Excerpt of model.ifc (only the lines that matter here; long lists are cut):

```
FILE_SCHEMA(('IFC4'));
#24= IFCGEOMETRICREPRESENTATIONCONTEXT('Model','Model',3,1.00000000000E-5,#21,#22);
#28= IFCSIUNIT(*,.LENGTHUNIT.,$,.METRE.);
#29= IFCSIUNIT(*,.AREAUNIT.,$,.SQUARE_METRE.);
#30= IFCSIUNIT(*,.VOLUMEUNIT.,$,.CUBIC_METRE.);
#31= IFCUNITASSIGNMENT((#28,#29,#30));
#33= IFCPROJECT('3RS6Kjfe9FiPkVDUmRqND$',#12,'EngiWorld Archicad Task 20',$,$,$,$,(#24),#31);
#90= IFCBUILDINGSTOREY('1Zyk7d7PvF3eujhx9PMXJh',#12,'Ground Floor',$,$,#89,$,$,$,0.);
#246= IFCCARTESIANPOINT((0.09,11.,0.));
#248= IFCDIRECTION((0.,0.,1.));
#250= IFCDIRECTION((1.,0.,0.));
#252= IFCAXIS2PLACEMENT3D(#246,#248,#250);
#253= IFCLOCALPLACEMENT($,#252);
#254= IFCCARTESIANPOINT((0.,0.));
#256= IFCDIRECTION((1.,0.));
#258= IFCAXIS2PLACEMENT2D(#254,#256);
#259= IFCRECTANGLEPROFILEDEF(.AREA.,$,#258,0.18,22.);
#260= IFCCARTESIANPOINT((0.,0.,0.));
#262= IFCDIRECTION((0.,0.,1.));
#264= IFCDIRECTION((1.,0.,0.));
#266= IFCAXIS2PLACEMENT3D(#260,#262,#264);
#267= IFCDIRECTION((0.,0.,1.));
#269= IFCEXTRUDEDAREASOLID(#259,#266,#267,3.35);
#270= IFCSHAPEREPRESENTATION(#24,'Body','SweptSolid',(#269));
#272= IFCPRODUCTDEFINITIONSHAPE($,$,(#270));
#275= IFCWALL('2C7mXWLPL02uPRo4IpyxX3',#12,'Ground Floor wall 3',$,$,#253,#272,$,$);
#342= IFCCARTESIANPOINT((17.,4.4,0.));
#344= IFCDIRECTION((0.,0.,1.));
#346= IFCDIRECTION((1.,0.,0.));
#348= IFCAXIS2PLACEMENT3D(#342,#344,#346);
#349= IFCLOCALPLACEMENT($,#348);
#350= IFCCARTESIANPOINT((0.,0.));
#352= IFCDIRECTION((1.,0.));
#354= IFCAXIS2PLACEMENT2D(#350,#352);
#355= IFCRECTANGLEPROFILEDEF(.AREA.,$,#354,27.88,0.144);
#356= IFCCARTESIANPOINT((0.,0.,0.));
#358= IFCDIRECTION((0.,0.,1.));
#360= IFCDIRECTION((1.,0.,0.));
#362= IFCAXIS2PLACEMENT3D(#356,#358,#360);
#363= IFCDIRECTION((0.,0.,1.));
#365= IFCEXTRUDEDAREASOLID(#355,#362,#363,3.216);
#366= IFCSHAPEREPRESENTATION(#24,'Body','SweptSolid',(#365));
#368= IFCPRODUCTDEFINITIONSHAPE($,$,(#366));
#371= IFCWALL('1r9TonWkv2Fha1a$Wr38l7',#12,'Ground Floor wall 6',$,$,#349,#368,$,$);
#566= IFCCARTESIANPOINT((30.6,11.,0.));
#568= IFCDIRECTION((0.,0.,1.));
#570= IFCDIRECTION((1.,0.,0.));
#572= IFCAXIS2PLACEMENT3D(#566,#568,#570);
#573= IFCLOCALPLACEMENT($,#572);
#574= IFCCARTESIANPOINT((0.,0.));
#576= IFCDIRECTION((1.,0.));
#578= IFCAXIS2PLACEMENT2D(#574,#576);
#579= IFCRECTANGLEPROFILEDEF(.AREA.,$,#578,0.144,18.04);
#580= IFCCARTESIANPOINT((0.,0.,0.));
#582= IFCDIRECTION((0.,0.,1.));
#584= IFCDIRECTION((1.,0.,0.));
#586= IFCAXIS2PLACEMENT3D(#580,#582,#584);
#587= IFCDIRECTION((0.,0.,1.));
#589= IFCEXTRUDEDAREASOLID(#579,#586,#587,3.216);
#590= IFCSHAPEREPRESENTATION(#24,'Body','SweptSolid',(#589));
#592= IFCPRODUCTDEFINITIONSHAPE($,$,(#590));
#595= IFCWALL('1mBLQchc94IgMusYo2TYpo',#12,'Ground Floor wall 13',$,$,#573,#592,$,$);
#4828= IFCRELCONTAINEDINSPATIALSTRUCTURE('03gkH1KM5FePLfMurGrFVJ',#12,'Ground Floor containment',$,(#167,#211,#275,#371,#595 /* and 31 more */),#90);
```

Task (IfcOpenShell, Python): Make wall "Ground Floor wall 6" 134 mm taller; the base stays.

```python
import ifcopenshell
import ifcopenshell.geom
import ifcopenshell.util.shape
import ifcopenshell.util.unit

model = ifcopenshell.open("model.ifc")
unit_scale = ifcopenshell.util.unit.calculate_unit_scale(model)
settings = ifcopenshell.geom.settings()


def volume(element):
    """Net volume in cubic metres, openings subtracted."""
    shape = ifcopenshell.geom.create_shape(settings, element)
    return ifcopenshell.util.shape.get_volume(shape.geometry)


wall = model.by_guid("1r9TonWkv2Fha1a$Wr38l7")
before = volume(wall)

body = next(r for r in wall.Representation.Representations if r.RepresentationIdentifier == "Body")
solid = body.Items[0]
old_height = solid.Depth
solid.Depth += 0.134 / unit_scale
after = volume(wall)

print(f"height {old_height:g} -> {solid.Depth:g}, volume {before:.3f} -> {after:.3f} m3")

model.write("model_v2.ifc")
```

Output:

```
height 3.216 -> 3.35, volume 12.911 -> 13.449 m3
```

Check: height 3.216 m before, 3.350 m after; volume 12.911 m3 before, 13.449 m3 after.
